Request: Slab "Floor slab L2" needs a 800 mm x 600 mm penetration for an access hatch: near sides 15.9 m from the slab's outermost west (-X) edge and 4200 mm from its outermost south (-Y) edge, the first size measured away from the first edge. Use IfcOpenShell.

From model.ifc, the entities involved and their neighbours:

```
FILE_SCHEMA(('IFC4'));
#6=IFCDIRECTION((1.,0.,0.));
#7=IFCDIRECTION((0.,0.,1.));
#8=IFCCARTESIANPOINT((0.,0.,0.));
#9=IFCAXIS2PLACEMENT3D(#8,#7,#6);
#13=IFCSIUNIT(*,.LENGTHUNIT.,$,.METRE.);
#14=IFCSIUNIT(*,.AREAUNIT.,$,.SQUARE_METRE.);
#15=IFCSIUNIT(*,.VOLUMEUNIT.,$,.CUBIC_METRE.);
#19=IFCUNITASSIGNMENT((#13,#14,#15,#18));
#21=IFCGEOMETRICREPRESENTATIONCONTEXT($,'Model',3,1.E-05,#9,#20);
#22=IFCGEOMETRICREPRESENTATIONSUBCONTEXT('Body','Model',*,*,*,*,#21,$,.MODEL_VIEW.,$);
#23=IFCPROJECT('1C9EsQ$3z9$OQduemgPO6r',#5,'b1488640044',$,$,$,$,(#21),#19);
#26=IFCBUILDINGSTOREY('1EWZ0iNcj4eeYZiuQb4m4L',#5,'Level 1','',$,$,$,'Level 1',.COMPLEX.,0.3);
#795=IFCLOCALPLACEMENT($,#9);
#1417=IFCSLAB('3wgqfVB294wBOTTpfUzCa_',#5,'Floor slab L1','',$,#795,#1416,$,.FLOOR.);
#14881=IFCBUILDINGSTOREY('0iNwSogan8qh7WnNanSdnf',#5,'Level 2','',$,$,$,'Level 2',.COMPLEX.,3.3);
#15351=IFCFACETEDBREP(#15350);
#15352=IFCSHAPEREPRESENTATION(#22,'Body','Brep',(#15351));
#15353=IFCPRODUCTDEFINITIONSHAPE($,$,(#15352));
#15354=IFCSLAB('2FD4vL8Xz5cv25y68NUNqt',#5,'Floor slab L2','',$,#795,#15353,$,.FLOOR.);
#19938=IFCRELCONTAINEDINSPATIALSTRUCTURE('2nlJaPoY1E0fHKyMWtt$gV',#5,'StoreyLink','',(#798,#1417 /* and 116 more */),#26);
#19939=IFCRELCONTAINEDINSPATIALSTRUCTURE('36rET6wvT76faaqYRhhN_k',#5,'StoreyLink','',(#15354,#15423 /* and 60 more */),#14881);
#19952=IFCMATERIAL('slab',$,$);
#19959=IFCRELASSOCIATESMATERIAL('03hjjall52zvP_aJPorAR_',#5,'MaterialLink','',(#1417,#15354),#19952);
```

```python
import numpy as np
import ifcopenshell
import ifcopenshell.api.feature
import ifcopenshell.api.geometry
import ifcopenshell.api.root
import ifcopenshell.geom
import ifcopenshell.util.placement
import ifcopenshell.util.representation
import ifcopenshell.util.shape
import ifcopenshell.util.unit

model = ifcopenshell.open("model.ifc")
unit_scale = ifcopenshell.util.unit.calculate_unit_scale(model)
settings = ifcopenshell.geom.settings()


def volume(element):
    """Net volume in cubic metres, openings subtracted."""
    shape = ifcopenshell.geom.create_shape(settings, element)
    return ifcopenshell.util.shape.get_volume(shape.geometry)


slab = model.by_guid("2FD4vL8Xz5cv25y68NUNqt")
before = volume(slab)

# Extent in the slab's own axes, in metres. The edges named are its -X and -Y sides.
slab_shape = ifcopenshell.geom.create_shape(settings, slab)
vertices = ifcopenshell.util.shape.get_vertices(slab_shape.geometry)
x_min, y_min, bottom = vertices.min(axis=0)
top = vertices[:, 2].max()

opening = ifcopenshell.api.root.create_entity(model, ifc_class="IfcOpeningElement", name="Access hatch opening", predefined_type="OPENING")
context = ifcopenshell.util.representation.get_context(model, "Model", "Body", "MODEL_VIEW")
width, depth = 0.8, 0.6
outline = [(0.0, 0.0), (width, 0.0), (width, depth), (0.0, depth), (0.0, 0.0)]
# Overshoot both faces by 50 mm so the cut is clean.
shape = ifcopenshell.api.geometry.add_slab_representation(
    model, context=context, depth=top - bottom + 0.1, polyline=outline
)
ifcopenshell.api.geometry.assign_representation(model, product=opening, representation=shape)

matrix = ifcopenshell.util.placement.get_local_placement(slab.ObjectPlacement)
matrix[:, 3] = matrix @ np.append(np.array([x_min + 15.9, y_min + 4.2, bottom - 0.05]) / unit_scale, 1.0)
ifcopenshell.api.geometry.edit_object_placement(model, product=opening, matrix=matrix, is_si=False)
ifcopenshell.api.feature.add_feature(model, feature=opening, element=slab)

after = volume(slab)

print(f"slab volume {before:.3f} -> {after:.3f} m3")

model.write("model-out.ifc")
```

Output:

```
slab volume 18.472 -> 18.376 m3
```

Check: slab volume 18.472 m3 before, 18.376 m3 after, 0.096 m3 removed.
